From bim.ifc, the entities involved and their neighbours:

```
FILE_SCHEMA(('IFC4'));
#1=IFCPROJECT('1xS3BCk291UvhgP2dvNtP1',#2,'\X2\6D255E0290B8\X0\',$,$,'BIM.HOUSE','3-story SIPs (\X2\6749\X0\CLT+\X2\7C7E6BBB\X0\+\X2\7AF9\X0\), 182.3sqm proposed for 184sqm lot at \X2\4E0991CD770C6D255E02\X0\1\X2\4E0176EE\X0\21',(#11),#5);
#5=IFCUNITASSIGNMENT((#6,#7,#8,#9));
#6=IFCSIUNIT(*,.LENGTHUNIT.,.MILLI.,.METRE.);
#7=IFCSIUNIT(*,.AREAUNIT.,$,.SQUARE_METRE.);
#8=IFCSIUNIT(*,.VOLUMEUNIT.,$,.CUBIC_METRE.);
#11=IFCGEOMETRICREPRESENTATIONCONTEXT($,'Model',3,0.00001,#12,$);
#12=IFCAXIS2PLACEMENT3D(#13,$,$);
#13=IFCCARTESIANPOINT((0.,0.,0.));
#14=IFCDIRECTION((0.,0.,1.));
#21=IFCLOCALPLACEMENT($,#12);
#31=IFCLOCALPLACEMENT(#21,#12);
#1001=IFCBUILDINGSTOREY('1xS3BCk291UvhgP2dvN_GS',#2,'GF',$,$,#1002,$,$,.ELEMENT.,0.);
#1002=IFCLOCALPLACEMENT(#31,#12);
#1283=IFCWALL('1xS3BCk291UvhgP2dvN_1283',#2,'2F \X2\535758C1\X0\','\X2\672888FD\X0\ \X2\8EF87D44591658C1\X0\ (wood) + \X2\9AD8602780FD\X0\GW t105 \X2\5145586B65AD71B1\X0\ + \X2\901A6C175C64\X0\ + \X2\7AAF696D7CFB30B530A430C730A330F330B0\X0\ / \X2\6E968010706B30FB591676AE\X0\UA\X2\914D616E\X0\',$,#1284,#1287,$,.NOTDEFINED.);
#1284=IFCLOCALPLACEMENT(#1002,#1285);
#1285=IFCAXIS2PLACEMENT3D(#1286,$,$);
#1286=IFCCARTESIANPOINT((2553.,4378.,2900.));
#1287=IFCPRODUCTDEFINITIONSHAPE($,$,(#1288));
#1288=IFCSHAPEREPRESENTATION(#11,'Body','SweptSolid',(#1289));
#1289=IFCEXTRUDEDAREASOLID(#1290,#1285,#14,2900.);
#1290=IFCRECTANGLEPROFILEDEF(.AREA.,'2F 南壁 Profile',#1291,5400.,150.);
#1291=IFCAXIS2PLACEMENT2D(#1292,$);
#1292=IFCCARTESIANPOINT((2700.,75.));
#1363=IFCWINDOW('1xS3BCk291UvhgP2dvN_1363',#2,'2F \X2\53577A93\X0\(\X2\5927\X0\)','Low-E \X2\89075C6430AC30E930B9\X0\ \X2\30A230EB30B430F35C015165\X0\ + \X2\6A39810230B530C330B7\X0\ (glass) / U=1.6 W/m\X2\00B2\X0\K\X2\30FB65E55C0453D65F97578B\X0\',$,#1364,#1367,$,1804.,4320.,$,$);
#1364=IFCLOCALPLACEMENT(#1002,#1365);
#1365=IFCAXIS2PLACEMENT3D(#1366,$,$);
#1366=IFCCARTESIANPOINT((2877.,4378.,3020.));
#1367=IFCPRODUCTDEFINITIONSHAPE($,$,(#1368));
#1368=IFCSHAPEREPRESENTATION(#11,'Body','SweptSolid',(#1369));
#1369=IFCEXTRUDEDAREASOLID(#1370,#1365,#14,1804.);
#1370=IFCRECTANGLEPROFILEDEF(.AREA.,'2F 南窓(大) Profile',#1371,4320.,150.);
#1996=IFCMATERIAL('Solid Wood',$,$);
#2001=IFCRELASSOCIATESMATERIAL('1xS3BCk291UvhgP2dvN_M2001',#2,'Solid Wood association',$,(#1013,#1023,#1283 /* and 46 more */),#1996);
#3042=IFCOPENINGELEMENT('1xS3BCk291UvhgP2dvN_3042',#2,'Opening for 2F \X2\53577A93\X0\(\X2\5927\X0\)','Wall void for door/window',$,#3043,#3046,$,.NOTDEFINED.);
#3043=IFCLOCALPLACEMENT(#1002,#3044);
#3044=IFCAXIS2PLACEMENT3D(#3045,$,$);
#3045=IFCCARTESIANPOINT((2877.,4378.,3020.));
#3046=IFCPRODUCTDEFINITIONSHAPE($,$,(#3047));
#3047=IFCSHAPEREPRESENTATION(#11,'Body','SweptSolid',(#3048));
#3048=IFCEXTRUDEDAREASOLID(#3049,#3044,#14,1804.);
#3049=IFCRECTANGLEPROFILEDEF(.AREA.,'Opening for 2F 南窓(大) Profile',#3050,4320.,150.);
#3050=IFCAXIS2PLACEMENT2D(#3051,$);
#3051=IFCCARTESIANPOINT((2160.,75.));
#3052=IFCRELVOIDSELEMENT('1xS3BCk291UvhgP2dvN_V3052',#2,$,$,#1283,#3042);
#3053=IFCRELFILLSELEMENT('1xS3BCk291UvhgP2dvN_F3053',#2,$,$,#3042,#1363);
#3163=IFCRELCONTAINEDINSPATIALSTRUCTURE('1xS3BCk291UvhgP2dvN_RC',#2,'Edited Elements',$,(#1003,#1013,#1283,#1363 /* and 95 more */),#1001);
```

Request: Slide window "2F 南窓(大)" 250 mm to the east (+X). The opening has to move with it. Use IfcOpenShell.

```python
import ifcopenshell
import ifcopenshell.api.geometry
import ifcopenshell.util.placement

model = ifcopenshell.open("bim.ifc")

window = model.by_id(1363)
opening = window.FillsVoids[0].RelatingOpeningElement
wall = opening.VoidsElements[0].RelatingBuildingElement

wall_matrix = ifcopenshell.util.placement.get_local_placement(wall.ObjectPlacement)
shift = wall_matrix[:3, 0] * 250.0
before = ifcopenshell.util.placement.get_local_placement(window.ObjectPlacement)[:3, 3].copy()

# The window is not placed relative to its opening, so move both.
for product in (opening, window):
    matrix = ifcopenshell.util.placement.get_local_placement(product.ObjectPlacement)
    matrix[:3, 3] += shift
    ifcopenshell.api.geometry.edit_object_placement(model, product=product, matrix=matrix, is_si=False)

after = ifcopenshell.util.placement.get_local_placement(window.ObjectPlacement)[:3, 3]
print("window moved by", (after - before).round(3) + 0.0)

model.write("bim-out.ifc")
```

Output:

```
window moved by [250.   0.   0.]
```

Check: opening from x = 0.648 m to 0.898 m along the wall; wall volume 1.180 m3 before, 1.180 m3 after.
